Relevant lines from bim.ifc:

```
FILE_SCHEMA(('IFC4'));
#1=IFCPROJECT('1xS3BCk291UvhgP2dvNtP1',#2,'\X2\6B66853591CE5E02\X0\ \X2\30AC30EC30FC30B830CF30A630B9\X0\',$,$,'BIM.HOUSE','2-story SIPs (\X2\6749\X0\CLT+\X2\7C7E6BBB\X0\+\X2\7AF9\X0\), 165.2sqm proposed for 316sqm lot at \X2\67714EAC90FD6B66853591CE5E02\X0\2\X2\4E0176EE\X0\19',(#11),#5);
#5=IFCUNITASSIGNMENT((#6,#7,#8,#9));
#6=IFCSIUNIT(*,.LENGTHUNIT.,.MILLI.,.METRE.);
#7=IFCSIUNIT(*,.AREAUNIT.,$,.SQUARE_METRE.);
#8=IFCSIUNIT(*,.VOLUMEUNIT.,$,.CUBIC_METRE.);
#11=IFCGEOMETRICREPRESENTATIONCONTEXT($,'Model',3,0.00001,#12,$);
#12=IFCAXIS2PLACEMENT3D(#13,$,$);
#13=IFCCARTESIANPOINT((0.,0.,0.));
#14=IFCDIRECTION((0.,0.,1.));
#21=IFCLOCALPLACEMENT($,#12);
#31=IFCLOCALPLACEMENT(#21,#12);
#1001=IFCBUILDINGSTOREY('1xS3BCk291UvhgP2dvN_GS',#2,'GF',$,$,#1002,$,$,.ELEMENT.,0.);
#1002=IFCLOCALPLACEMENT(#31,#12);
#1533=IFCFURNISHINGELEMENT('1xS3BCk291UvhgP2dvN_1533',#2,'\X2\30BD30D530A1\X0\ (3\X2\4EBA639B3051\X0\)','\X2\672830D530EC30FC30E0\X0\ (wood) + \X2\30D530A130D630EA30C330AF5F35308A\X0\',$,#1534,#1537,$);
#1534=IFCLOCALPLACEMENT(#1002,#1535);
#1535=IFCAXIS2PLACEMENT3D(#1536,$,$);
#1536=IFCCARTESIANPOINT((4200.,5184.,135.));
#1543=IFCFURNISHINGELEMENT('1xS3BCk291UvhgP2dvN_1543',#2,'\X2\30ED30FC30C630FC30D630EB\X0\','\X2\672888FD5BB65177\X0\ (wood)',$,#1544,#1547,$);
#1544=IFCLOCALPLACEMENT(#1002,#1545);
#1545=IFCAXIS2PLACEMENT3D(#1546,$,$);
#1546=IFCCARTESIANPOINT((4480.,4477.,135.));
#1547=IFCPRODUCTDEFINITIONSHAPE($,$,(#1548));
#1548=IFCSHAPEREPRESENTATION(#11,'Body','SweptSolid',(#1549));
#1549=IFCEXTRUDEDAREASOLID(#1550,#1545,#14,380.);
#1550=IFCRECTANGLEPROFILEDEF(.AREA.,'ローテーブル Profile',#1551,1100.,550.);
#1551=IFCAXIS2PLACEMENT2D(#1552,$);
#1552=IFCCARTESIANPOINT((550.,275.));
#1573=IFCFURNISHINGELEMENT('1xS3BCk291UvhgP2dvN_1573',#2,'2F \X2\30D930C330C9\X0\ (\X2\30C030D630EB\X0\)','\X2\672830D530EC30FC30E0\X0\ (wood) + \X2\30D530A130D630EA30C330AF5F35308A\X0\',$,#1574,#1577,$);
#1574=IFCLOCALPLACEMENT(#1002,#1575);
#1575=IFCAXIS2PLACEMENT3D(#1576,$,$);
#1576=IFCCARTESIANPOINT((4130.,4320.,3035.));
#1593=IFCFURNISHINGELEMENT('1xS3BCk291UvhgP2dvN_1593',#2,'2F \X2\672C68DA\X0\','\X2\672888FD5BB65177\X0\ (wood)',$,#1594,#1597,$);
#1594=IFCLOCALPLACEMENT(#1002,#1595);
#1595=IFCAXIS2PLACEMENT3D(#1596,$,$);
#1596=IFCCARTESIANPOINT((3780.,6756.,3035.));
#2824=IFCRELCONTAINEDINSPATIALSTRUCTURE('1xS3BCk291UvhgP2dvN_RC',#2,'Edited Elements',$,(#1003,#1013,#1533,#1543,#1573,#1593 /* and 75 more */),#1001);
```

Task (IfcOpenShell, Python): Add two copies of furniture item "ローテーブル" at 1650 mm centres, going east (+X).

```python
import numpy as np
import ifcopenshell
import ifcopenshell.api.geometry
import ifcopenshell.api.root
import ifcopenshell.util.element
import ifcopenshell.util.placement
import ifcopenshell.util.unit

model = ifcopenshell.open("bim.ifc")
unit_scale = ifcopenshell.util.unit.calculate_unit_scale(model)


def reuse_history(source, copy):
    """copy_class also copies each property set's owner history, people and application; keep the originals."""
    for rel in copy.IsDefinedBy:
        if rel.is_a("IfcRelDefinesByProperties") and (history := rel.RelatingPropertyDefinition.OwnerHistory):
            rel.RelatingPropertyDefinition.OwnerHistory = source.OwnerHistory
            ifcopenshell.util.element.remove_deep2(model, history)


source = model.by_guid("1xS3BCk291UvhgP2dvN_1543")
base = ifcopenshell.util.placement.get_local_placement(source.ObjectPlacement)
step = np.array([1.0, 0.0, 0.0]) * 1.65 / unit_scale

for i in range(1, 3):
    copy = ifcopenshell.api.root.copy_class(model, product=source)
    copy.Representation = ifcopenshell.util.element.copy_deep(
        model, source.Representation, exclude=["IfcGeometricRepresentationContext", "IfcRepresentationMap"]
    )
    reuse_history(source, copy)
    matrix = base.copy()
    matrix[:3, 3] += i * step
    print("added at", matrix[:3, 3].round(3) + 0.0)
    ifcopenshell.api.geometry.edit_object_placement(model, product=copy, matrix=matrix, is_si=False)

model.write("bim_edited.ifc")
```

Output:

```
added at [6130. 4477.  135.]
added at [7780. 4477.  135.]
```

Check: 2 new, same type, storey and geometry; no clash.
